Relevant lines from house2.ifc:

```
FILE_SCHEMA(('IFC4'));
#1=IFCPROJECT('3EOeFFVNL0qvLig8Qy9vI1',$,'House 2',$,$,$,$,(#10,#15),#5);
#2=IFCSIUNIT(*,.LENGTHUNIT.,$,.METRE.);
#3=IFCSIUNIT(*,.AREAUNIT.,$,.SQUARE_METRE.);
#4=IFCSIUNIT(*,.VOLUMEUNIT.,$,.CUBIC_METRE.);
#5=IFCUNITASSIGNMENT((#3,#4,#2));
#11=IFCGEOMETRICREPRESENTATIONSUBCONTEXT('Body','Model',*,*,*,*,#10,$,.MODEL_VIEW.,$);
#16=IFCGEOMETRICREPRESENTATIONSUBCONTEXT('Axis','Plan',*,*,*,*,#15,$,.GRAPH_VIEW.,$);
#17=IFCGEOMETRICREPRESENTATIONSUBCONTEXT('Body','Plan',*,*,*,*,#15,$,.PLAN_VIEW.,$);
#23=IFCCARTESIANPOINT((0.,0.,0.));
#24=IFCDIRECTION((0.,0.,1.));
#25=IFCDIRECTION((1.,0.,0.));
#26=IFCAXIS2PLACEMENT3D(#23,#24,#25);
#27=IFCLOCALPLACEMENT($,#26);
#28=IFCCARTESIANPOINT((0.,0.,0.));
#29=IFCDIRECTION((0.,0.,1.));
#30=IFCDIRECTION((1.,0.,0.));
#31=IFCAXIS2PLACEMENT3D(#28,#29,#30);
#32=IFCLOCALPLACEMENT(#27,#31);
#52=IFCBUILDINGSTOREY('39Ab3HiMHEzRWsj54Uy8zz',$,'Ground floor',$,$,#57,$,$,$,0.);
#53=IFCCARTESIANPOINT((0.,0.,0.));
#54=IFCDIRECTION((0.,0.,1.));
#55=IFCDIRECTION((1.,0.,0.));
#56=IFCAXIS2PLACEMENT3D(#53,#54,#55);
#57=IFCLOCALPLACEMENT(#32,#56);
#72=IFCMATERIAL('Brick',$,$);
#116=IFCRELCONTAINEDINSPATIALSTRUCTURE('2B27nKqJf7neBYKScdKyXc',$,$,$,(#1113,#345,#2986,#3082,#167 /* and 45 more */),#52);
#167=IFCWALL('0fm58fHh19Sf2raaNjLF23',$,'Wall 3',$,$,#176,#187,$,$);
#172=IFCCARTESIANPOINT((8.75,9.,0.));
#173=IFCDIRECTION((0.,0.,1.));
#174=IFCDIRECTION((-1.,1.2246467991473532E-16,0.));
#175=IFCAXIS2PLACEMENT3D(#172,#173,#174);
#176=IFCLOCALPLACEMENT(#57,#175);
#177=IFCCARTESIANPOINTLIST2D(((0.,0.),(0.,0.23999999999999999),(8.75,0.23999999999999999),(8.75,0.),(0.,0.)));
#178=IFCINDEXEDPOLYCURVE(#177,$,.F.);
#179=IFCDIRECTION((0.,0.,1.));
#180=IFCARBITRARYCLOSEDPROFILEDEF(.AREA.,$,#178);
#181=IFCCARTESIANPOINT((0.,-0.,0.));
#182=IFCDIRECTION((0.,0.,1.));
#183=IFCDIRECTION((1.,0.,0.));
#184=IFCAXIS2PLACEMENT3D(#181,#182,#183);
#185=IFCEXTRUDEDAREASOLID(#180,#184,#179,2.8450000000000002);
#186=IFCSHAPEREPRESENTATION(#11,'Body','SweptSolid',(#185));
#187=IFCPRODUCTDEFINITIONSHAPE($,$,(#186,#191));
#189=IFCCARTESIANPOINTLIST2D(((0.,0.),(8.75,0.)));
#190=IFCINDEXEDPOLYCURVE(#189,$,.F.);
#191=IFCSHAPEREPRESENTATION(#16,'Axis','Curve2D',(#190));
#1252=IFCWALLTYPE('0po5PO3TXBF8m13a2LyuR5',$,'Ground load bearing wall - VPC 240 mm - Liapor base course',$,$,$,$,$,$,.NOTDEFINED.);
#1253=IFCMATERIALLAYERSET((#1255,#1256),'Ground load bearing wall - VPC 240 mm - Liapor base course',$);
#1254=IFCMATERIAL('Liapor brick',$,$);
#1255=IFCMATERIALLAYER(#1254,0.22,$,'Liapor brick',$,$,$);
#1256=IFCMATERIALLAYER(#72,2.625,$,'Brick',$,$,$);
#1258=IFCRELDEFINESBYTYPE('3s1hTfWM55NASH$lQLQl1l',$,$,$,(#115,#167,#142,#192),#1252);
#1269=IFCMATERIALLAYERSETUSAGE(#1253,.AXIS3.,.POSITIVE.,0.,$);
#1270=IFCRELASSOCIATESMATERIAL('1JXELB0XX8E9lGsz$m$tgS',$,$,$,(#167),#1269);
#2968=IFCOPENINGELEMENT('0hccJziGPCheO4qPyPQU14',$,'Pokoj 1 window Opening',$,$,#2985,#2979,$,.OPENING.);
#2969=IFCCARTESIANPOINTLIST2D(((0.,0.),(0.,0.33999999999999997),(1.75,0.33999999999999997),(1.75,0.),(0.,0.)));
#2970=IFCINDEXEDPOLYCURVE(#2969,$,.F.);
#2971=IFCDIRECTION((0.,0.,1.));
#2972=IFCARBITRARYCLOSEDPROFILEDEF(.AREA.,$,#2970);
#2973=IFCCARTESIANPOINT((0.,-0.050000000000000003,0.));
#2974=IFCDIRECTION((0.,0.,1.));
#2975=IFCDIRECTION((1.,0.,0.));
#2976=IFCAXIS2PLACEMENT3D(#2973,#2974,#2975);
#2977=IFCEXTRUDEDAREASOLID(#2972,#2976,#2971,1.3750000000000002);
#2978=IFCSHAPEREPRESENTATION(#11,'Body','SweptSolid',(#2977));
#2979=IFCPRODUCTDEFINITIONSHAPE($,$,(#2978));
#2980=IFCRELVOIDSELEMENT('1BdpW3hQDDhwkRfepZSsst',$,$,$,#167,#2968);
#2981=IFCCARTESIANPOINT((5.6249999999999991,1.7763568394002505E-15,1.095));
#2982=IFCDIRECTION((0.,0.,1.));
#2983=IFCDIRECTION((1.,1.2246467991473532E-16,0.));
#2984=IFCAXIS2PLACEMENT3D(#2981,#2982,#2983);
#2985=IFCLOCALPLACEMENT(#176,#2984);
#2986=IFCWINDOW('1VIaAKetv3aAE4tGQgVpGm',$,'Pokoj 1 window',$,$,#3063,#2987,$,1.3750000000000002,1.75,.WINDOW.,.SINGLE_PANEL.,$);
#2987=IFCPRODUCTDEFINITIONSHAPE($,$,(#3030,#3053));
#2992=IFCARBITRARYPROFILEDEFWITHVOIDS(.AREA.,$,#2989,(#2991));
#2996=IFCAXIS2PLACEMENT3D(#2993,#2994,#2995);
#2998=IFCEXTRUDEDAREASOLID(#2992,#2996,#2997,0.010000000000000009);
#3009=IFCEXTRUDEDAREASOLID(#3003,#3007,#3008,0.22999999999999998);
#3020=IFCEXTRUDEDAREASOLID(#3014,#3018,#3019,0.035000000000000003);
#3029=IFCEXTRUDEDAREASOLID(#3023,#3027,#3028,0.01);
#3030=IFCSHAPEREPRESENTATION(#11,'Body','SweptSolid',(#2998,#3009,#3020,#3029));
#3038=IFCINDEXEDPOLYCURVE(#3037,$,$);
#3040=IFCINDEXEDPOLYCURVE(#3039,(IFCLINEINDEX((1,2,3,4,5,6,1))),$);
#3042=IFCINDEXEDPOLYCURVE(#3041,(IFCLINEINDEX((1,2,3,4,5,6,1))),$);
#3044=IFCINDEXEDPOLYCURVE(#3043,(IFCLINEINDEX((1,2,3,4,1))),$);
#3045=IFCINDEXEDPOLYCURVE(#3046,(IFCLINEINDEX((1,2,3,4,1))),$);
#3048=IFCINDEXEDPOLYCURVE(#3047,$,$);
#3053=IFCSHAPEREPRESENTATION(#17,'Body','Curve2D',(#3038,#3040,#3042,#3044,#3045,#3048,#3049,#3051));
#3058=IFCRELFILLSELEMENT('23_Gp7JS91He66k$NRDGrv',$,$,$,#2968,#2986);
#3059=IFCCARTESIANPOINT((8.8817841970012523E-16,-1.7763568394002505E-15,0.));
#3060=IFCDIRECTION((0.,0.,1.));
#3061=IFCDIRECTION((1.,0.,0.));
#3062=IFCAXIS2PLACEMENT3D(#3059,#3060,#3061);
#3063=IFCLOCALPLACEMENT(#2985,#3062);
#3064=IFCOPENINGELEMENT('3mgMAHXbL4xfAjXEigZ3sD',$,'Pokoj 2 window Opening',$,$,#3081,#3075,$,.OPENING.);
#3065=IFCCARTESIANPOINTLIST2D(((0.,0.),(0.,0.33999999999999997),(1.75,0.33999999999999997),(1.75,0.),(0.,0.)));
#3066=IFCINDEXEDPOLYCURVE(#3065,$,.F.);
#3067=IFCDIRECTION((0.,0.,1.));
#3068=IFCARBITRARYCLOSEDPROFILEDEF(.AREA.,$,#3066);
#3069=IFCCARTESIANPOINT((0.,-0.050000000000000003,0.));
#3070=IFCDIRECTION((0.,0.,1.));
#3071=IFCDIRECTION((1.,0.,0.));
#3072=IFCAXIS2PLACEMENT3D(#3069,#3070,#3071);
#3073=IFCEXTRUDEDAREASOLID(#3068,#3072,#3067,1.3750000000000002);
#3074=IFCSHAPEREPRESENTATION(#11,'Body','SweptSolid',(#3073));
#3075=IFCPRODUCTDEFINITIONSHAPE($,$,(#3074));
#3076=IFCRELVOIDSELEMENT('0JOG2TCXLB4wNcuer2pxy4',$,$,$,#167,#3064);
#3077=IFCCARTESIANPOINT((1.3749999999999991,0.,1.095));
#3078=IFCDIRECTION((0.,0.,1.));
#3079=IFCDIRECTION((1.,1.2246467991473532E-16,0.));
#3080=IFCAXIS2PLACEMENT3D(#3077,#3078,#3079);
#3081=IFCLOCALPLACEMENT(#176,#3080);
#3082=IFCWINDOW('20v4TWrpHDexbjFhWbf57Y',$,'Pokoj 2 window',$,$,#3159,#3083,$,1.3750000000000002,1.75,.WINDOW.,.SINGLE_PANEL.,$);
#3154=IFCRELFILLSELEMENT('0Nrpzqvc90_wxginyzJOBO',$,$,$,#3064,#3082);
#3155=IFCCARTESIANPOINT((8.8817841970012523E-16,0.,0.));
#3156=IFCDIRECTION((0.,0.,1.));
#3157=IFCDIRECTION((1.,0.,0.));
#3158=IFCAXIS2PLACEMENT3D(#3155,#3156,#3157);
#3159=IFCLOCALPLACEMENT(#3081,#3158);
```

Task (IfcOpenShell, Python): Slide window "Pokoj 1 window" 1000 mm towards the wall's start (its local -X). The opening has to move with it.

```python
import ifcopenshell
import ifcopenshell.api.geometry
import ifcopenshell.util.placement

model = ifcopenshell.open("house2.ifc")

window = model.by_guid("1VIaAKetv3aAE4tGQgVpGm")
opening = window.FillsVoids[0].RelatingOpeningElement
wall = opening.VoidsElements[0].RelatingBuildingElement

wall_matrix = ifcopenshell.util.placement.get_local_placement(wall.ObjectPlacement)
shift = wall_matrix[:3, 0] * -1.0
before = ifcopenshell.util.placement.get_local_placement(window.ObjectPlacement)[:3, 3].copy()

# The window is placed relative to its opening, so it follows when the opening moves.
matrix = ifcopenshell.util.placement.get_local_placement(opening.ObjectPlacement)
matrix[:3, 3] += shift
ifcopenshell.api.geometry.edit_object_placement(
    model, product=opening, matrix=matrix, is_si=False, should_transform_children=True
)

after = ifcopenshell.util.placement.get_local_placement(window.ObjectPlacement)[:3, 3]
print("window moved by", (after - before).round(3) + 0.0)

model.write("house2-out.ifc")
```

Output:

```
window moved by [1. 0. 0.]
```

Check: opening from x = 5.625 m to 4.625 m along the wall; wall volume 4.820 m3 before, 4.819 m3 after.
